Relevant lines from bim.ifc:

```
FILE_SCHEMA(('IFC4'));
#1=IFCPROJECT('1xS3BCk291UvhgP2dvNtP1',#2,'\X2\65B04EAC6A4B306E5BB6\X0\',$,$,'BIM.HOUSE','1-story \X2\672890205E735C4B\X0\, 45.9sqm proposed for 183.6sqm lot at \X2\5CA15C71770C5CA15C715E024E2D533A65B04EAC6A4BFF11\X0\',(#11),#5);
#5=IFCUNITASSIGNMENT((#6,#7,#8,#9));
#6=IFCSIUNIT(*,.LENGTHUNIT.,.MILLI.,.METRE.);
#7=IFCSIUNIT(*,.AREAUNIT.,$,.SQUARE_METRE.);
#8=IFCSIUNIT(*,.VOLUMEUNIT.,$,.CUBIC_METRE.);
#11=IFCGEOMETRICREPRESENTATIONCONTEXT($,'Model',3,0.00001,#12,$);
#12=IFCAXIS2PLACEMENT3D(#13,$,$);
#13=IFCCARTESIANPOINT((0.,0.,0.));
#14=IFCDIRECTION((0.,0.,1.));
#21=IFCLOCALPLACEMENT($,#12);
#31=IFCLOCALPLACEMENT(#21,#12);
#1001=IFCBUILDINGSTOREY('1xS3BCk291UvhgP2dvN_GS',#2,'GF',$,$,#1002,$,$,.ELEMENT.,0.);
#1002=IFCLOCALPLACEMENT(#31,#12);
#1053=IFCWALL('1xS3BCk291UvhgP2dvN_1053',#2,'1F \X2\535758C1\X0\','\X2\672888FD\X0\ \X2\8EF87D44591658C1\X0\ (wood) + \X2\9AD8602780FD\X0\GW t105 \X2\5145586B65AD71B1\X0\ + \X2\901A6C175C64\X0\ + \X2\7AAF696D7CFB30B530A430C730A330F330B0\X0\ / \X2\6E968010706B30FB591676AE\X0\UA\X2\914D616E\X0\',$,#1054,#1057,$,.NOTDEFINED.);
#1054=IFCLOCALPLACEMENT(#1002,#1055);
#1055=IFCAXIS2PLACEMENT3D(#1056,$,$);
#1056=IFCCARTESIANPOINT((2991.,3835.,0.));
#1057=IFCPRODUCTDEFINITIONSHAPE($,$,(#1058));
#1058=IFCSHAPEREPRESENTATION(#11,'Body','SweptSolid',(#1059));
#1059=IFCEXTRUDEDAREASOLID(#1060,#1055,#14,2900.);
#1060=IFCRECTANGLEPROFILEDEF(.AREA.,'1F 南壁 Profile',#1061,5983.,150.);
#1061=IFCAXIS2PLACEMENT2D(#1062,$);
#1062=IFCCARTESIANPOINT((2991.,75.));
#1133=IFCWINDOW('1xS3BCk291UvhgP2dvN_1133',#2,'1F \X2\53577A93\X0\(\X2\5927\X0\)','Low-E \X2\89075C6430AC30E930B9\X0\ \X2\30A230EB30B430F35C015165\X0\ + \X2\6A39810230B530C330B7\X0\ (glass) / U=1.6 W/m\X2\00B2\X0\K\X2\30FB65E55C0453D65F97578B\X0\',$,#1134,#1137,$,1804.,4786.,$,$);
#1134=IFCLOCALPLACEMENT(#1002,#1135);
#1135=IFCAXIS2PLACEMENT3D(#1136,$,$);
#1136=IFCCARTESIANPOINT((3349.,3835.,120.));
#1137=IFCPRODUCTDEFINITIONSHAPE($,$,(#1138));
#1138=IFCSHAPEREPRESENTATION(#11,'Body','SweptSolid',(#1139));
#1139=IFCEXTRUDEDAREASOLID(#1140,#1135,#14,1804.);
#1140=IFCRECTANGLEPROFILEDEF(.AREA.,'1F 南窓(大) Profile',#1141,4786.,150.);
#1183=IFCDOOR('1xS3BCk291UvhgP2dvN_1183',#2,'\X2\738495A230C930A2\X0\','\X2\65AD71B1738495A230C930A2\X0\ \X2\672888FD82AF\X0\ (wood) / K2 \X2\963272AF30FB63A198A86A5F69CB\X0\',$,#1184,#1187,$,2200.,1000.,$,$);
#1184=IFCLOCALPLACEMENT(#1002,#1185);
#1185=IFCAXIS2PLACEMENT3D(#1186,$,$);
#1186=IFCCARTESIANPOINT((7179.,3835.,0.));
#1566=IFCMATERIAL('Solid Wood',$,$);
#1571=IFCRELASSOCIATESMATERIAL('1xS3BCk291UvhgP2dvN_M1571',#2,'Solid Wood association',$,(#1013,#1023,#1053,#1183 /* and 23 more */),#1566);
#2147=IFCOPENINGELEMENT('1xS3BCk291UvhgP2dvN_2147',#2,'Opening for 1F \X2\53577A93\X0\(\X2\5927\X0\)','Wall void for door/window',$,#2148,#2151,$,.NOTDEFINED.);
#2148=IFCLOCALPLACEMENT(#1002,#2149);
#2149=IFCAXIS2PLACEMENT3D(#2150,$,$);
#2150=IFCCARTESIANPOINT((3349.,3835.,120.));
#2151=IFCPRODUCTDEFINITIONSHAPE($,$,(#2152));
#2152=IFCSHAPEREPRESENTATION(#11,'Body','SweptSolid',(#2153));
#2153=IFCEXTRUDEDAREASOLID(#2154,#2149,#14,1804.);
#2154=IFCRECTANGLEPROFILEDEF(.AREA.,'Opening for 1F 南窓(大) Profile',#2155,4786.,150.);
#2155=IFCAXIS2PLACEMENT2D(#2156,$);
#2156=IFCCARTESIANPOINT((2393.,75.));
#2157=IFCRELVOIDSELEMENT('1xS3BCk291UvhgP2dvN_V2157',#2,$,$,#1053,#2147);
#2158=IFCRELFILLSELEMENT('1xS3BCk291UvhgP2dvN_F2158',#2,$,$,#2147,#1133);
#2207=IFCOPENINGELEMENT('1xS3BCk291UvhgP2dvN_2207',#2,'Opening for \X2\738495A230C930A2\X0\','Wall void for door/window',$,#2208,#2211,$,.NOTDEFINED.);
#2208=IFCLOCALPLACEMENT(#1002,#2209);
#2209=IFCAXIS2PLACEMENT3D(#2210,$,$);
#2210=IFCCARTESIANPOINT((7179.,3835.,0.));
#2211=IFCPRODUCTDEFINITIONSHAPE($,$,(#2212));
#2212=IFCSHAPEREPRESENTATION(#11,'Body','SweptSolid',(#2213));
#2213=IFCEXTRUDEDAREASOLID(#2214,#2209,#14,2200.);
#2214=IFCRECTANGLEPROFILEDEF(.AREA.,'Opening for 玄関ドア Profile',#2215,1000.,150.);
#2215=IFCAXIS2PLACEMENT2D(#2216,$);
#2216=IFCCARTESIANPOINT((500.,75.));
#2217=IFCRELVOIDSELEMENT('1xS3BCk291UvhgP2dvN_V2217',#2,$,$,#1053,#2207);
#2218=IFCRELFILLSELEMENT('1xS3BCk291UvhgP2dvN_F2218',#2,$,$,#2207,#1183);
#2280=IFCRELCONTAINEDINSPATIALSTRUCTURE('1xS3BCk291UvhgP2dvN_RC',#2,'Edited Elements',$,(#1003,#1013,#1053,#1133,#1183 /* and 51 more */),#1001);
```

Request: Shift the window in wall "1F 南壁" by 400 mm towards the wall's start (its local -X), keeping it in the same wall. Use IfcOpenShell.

```python
import ifcopenshell
import ifcopenshell.api.geometry
import ifcopenshell.util.placement

model = ifcopenshell.open("bim.ifc")

window = model.by_guid("1xS3BCk291UvhgP2dvN_1133")
opening = window.FillsVoids[0].RelatingOpeningElement
wall = opening.VoidsElements[0].RelatingBuildingElement

wall_matrix = ifcopenshell.util.placement.get_local_placement(wall.ObjectPlacement)
shift = wall_matrix[:3, 0] * -400.0
before = ifcopenshell.util.placement.get_local_placement(window.ObjectPlacement)[:3, 3].copy()

# The window is not placed relative to its opening, so move both.
for product in (opening, window):
    matrix = ifcopenshell.util.placement.get_local_placement(product.ObjectPlacement)
    matrix[:3, 3] += shift
    ifcopenshell.api.geometry.edit_object_placement(model, product=product, matrix=matrix, is_si=False)

after = ifcopenshell.util.placement.get_local_placement(window.ObjectPlacement)[:3, 3]
print("window moved by", (after - before).round(3) + 0.0)

model.write("bim_v2.ifc")
```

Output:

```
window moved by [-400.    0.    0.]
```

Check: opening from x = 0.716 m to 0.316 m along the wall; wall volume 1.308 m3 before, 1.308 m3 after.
